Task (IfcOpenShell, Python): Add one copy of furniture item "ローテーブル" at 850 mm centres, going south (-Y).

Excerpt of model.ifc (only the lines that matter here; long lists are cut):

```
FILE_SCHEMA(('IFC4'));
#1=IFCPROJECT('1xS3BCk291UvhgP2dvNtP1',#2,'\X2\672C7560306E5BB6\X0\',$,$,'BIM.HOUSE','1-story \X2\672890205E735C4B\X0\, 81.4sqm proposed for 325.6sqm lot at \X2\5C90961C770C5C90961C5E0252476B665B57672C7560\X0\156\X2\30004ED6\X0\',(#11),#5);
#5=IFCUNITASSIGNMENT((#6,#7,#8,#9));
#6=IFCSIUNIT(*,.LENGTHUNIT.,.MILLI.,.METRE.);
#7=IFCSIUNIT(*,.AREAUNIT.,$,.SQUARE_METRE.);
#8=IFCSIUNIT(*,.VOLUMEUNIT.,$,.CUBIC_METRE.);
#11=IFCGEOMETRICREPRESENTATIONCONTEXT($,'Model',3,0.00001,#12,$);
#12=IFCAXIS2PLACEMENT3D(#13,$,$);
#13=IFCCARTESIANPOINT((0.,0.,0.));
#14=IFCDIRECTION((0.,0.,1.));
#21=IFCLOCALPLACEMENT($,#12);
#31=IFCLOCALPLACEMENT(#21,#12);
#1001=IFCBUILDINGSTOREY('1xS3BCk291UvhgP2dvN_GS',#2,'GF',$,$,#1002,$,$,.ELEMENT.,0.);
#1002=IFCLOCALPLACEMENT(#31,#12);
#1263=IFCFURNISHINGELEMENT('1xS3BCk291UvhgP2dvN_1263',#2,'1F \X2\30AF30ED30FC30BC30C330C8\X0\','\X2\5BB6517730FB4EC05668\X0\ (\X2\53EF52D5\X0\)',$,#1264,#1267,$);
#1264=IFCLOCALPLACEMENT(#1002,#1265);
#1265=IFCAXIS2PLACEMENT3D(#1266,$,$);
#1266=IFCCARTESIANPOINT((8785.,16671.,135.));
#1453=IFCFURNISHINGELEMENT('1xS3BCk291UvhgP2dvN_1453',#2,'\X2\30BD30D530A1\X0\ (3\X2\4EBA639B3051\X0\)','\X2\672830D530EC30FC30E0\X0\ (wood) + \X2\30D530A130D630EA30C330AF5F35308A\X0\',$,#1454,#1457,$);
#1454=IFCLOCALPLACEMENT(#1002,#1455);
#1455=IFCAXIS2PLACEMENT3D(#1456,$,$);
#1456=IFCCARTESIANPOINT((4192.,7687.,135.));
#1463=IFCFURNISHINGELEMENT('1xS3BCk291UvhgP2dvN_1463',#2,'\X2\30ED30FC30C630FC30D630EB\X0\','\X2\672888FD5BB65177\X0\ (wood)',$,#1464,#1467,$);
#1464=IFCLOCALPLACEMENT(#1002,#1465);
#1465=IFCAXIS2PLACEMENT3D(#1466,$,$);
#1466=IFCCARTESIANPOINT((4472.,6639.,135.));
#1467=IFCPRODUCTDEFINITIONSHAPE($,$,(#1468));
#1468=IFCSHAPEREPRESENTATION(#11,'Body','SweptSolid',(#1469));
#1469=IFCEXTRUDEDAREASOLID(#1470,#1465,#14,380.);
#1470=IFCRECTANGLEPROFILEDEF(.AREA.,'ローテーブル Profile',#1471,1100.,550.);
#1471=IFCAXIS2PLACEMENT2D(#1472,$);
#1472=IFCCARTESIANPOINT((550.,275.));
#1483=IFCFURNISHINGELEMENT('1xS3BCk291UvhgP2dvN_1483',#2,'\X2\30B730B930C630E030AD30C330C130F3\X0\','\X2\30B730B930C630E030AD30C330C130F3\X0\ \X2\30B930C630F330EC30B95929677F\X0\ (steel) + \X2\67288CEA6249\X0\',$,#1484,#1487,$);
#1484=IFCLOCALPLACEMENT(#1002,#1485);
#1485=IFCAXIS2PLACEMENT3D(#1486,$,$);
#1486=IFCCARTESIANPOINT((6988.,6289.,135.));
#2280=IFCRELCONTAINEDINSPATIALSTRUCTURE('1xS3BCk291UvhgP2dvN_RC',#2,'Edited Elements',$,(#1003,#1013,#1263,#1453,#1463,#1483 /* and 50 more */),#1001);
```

```python
import numpy as np
import ifcopenshell
import ifcopenshell.api.geometry
import ifcopenshell.api.root
import ifcopenshell.util.element
import ifcopenshell.util.placement
import ifcopenshell.util.unit

model = ifcopenshell.open("model.ifc")
unit_scale = ifcopenshell.util.unit.calculate_unit_scale(model)


def reuse_history(source, copy):
    """copy_class also copies each property set's owner history, people and application; keep the originals."""
    for rel in copy.IsDefinedBy:
        if rel.is_a("IfcRelDefinesByProperties") and (history := rel.RelatingPropertyDefinition.OwnerHistory):
            rel.RelatingPropertyDefinition.OwnerHistory = source.OwnerHistory
            ifcopenshell.util.element.remove_deep2(model, history)


source = model.by_guid("1xS3BCk291UvhgP2dvN_1463")
base = ifcopenshell.util.placement.get_local_placement(source.ObjectPlacement)
step = np.array([0.0, -1.0, 0.0]) * 0.85 / unit_scale

for i in range(1, 2):
    copy = ifcopenshell.api.root.copy_class(model, product=source)
    copy.Representation = ifcopenshell.util.element.copy_deep(
        model, source.Representation, exclude=["IfcGeometricRepresentationContext", "IfcRepresentationMap"]
    )
    reuse_history(source, copy)
    matrix = base.copy()
    matrix[:3, 3] += i * step
    print("added at", matrix[:3, 3].round(3) + 0.0)
    ifcopenshell.api.geometry.edit_object_placement(model, product=copy, matrix=matrix, is_si=False)

model.write("model_updated.ifc")
```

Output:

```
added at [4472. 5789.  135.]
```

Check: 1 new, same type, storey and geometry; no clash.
